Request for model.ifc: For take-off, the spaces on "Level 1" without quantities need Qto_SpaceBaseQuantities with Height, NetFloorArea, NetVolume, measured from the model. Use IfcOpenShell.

First a look at what the model holds.

```python
import ifcopenshell
import ifcopenshell.util.element
import ifcopenshell.util.unit

model = ifcopenshell.open("model.ifc")
print(model.schema)
for unit_type in ("LENGTHUNIT", "AREAUNIT", "VOLUMEUNIT"):
    print(unit_type, ifcopenshell.util.unit.calculate_unit_scale(model, unit_type))
storey = next(s for s in model.by_type("IfcBuildingStorey") if s.Name == "Level 1")
spaces = [e for e in ifcopenshell.util.element.get_decomposition(storey) if e.is_a("IfcSpace")]
for e in sorted(spaces, key=lambda e: e.id()):
    print(e.id(), e.is_a(), e.Name, list(ifcopenshell.util.element.get_psets(e, qtos_only=True)), sep=" | ")
```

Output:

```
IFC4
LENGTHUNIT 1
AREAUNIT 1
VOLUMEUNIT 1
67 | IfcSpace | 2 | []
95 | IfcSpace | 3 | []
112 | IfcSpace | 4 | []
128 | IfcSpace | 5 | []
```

```python
import ifcopenshell
import ifcopenshell.api.pset
import ifcopenshell.geom
import ifcopenshell.util.element
import ifcopenshell.util.shape
import ifcopenshell.util.unit

model = ifcopenshell.open("model.ifc")
unit_scale = ifcopenshell.util.unit.calculate_unit_scale(model)
area_scale = ifcopenshell.util.unit.calculate_unit_scale(model, "AREAUNIT")
volume_scale = ifcopenshell.util.unit.calculate_unit_scale(model, "VOLUMEUNIT")
settings = ifcopenshell.geom.settings()

storey = next(s for s in model.by_type("IfcBuildingStorey") if s.Name == "Level 1")
spaces = [e for e in ifcopenshell.util.element.get_decomposition(storey) if e.is_a("IfcSpace")]

for e in sorted(spaces, key=lambda e: e.id()):
    if ifcopenshell.util.element.get_psets(e, qtos_only=True, should_inherit=False):
        continue
    # Geometry comes back in metres, in the element's own axes.
    shape = ifcopenshell.geom.create_shape(settings, e)
    values = {
        "Height": ifcopenshell.util.shape.get_z(shape.geometry) / unit_scale,
        "NetFloorArea": ifcopenshell.util.shape.get_footprint_area(shape.geometry) / area_scale,
        "NetVolume": ifcopenshell.util.shape.get_volume(shape.geometry) / volume_scale,
    }
    qto = ifcopenshell.api.pset.add_qto(model, product=e, name="Qto_SpaceBaseQuantities")
    ifcopenshell.api.pset.edit_qto(model, qto=qto, properties=values)
    print(e.id(), {k: round(v, 3) for k, v in values.items()})

model.write("model_rev.ifc")
```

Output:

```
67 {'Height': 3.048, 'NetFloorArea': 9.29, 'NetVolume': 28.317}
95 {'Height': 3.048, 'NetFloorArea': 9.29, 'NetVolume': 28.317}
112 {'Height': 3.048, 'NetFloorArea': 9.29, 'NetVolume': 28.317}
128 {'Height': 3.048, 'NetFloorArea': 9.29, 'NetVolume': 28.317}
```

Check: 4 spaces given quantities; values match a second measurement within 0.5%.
